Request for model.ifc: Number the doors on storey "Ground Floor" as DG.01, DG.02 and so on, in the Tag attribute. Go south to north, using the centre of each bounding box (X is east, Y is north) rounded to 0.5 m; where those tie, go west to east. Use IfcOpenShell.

First a look at what the model holds.

```python
import ifcopenshell
import ifcopenshell.util.element
import ifcopenshell.util.placement

model = ifcopenshell.open("model.ifc")
print(model.schema)
storey = next(s for s in model.by_type("IfcBuildingStorey") if s.Name == "Ground Floor")
doors = [e for e in ifcopenshell.util.element.get_decomposition(storey) if e.is_a("IfcDoor")]
for e in sorted(doors, key=lambda e: e.id()):
    origin = ifcopenshell.util.placement.get_local_placement(e.ObjectPlacement)[:3, 3]
    print(e.id(), e.Tag, e.Name, origin.round(2) + 0.0, sep=" | ")
```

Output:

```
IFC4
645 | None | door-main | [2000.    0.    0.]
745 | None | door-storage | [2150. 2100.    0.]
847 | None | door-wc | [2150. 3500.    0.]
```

```python
import ifcopenshell
import ifcopenshell.geom
import ifcopenshell.util.element
import ifcopenshell.util.shape

model = ifcopenshell.open("model.ifc")
settings = ifcopenshell.geom.settings()
settings.set("use-world-coords", True)


def centre(element):
    shape = ifcopenshell.geom.create_shape(settings, element)
    return ifcopenshell.util.shape.get_bbox_centroid(shape.geometry)


storey = next(s for s in model.by_type("IfcBuildingStorey") if s.Name == "Ground Floor")
doors = [e for e in ifcopenshell.util.element.get_decomposition(storey) if e.is_a("IfcDoor")]

# Insertion points can sit at a corner or the storey origin, so sort by the geometry (in metres).
centres = {e: centre(e) for e in doors}
doors.sort(key=lambda e: (round(centres[e][1] / 0.5), centres[e][0]))

for i, e in enumerate(doors, start=1):
    number = f"DG.{i:02d}"
    e.Tag = number
    print(e.id(), number)

model.write("model_updated.ifc")
```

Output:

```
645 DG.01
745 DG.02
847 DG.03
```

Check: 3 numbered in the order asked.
